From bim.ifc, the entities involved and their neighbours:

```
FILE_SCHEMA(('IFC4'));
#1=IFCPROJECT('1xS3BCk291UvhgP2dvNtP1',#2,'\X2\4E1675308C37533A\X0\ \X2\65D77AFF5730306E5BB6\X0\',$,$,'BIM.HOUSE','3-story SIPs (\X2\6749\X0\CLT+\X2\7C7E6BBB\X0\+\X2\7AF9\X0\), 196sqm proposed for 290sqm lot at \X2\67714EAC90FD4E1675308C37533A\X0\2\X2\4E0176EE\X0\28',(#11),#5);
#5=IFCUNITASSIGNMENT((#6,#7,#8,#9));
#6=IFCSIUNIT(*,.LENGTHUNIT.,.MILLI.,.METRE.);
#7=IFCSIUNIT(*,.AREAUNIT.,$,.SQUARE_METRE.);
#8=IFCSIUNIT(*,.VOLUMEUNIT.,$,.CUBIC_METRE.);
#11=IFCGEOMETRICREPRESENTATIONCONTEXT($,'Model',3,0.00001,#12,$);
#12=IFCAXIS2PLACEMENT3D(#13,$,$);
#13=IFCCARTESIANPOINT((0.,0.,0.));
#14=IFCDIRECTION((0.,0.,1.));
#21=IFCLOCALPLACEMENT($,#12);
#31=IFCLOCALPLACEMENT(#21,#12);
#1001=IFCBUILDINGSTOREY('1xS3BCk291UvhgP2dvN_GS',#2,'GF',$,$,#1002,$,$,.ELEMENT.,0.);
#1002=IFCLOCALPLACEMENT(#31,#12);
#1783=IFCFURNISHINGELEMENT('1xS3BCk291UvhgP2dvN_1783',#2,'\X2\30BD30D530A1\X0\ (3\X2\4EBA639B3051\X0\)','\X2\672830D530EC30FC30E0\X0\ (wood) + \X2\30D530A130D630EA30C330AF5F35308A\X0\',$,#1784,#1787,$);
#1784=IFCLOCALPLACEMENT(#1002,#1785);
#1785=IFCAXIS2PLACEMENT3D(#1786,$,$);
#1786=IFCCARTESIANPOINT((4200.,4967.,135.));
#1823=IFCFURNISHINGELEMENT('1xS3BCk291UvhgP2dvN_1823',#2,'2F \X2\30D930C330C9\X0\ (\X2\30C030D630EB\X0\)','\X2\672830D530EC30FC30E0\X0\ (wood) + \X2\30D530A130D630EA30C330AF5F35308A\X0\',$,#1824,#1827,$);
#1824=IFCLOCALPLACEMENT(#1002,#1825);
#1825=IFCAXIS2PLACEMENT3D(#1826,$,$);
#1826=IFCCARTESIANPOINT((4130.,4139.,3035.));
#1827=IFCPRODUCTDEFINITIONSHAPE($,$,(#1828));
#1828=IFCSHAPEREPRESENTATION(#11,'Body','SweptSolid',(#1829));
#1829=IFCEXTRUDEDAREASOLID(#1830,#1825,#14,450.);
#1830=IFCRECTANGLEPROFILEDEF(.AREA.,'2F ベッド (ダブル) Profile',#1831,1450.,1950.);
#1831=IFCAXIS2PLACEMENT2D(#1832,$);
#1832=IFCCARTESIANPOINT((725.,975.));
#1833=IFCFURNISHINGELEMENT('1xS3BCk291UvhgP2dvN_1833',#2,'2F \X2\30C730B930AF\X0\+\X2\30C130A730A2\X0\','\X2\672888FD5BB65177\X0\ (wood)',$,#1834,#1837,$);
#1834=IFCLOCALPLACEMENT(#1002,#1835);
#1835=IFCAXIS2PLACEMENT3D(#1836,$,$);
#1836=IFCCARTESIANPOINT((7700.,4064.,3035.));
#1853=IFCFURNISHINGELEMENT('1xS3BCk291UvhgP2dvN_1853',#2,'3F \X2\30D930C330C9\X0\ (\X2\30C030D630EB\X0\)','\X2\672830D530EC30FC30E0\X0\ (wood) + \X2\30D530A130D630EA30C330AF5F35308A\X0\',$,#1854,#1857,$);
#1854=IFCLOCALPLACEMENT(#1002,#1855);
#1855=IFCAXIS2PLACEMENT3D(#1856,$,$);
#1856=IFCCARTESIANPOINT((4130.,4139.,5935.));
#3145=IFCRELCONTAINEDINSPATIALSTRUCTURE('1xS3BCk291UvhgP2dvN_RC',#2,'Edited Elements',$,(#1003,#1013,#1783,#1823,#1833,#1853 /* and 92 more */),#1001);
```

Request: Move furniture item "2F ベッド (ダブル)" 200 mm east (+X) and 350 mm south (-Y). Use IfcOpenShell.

```python
import ifcopenshell
import ifcopenshell.api.geometry
import ifcopenshell.util.placement
import ifcopenshell.util.unit

model = ifcopenshell.open("bim.ifc")
unit_scale = ifcopenshell.util.unit.calculate_unit_scale(model)

item = model.by_id(1823)
matrix = ifcopenshell.util.placement.get_local_placement(item.ObjectPlacement)
matrix[0, 3] += 0.2 / unit_scale
matrix[1, 3] -= 0.35 / unit_scale
ifcopenshell.api.geometry.edit_object_placement(model, product=item, matrix=matrix, is_si=False)

print(ifcopenshell.util.placement.get_local_placement(item.ObjectPlacement).round(3) + 0.0)

model.write("bim_v2.ifc")
```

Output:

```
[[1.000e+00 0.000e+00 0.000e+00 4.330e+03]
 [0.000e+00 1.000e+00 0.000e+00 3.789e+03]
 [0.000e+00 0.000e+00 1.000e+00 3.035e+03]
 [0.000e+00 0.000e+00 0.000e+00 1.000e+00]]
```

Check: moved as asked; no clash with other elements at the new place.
